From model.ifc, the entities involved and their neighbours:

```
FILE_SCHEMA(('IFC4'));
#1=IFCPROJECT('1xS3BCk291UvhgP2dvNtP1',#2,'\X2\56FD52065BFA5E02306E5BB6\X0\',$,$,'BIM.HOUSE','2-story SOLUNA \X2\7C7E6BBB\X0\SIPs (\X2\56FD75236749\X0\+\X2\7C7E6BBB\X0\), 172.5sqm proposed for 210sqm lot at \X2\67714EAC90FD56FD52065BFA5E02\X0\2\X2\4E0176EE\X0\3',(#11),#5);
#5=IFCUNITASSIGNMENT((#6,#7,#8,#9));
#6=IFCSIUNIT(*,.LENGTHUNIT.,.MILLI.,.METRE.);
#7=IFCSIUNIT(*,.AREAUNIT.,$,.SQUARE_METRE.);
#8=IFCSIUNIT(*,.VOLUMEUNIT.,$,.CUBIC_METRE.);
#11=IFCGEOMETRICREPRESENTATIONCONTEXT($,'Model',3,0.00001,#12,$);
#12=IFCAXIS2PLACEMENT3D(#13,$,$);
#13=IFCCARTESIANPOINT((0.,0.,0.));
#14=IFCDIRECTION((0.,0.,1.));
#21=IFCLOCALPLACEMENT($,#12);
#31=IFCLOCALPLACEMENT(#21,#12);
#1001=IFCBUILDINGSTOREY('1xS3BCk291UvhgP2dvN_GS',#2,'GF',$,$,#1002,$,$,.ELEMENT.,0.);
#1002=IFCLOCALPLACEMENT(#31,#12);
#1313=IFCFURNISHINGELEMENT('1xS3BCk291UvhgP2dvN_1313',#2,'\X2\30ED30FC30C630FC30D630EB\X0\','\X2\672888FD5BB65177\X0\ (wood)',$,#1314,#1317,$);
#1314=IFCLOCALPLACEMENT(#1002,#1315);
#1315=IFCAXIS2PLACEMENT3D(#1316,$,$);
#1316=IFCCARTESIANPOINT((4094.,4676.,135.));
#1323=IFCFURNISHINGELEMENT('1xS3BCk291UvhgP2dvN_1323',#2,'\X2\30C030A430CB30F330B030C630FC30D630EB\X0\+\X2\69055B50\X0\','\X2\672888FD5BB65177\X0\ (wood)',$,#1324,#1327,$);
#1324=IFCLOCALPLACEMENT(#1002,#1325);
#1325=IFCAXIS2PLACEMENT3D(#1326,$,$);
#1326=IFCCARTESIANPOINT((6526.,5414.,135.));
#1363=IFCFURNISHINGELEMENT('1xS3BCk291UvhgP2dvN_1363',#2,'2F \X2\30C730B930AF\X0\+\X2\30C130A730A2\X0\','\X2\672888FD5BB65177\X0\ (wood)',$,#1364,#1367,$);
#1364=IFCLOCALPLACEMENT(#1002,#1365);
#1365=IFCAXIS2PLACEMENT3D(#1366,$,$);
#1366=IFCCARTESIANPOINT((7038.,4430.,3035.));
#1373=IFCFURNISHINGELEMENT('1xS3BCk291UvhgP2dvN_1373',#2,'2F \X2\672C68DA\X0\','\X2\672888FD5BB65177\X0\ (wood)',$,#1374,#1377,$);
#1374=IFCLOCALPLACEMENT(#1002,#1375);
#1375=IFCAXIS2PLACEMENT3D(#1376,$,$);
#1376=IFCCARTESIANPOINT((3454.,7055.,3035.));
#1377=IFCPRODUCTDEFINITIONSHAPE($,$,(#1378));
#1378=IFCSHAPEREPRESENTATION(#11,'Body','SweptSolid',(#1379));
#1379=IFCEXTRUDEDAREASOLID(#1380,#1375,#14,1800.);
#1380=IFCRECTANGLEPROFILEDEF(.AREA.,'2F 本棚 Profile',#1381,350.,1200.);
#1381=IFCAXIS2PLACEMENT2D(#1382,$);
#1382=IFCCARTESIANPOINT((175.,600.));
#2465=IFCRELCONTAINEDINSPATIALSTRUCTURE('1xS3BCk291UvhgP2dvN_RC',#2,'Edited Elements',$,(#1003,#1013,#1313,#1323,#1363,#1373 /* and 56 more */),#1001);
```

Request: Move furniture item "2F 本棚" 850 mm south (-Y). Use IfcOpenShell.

```python
import ifcopenshell
import ifcopenshell.api.geometry
import ifcopenshell.util.placement
import ifcopenshell.util.unit

model = ifcopenshell.open("model.ifc")
unit_scale = ifcopenshell.util.unit.calculate_unit_scale(model)

item = model.by_guid("1xS3BCk291UvhgP2dvN_1373")
matrix = ifcopenshell.util.placement.get_local_placement(item.ObjectPlacement)
matrix[1, 3] -= 0.85 / unit_scale
ifcopenshell.api.geometry.edit_object_placement(model, product=item, matrix=matrix, is_si=False)

print(ifcopenshell.util.placement.get_local_placement(item.ObjectPlacement).round(3) + 0.0)

model.write("model_edited.ifc")
```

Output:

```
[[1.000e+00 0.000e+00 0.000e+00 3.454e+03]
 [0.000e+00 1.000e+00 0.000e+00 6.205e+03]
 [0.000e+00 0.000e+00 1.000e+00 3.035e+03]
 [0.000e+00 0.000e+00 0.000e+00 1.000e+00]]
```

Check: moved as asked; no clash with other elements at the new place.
